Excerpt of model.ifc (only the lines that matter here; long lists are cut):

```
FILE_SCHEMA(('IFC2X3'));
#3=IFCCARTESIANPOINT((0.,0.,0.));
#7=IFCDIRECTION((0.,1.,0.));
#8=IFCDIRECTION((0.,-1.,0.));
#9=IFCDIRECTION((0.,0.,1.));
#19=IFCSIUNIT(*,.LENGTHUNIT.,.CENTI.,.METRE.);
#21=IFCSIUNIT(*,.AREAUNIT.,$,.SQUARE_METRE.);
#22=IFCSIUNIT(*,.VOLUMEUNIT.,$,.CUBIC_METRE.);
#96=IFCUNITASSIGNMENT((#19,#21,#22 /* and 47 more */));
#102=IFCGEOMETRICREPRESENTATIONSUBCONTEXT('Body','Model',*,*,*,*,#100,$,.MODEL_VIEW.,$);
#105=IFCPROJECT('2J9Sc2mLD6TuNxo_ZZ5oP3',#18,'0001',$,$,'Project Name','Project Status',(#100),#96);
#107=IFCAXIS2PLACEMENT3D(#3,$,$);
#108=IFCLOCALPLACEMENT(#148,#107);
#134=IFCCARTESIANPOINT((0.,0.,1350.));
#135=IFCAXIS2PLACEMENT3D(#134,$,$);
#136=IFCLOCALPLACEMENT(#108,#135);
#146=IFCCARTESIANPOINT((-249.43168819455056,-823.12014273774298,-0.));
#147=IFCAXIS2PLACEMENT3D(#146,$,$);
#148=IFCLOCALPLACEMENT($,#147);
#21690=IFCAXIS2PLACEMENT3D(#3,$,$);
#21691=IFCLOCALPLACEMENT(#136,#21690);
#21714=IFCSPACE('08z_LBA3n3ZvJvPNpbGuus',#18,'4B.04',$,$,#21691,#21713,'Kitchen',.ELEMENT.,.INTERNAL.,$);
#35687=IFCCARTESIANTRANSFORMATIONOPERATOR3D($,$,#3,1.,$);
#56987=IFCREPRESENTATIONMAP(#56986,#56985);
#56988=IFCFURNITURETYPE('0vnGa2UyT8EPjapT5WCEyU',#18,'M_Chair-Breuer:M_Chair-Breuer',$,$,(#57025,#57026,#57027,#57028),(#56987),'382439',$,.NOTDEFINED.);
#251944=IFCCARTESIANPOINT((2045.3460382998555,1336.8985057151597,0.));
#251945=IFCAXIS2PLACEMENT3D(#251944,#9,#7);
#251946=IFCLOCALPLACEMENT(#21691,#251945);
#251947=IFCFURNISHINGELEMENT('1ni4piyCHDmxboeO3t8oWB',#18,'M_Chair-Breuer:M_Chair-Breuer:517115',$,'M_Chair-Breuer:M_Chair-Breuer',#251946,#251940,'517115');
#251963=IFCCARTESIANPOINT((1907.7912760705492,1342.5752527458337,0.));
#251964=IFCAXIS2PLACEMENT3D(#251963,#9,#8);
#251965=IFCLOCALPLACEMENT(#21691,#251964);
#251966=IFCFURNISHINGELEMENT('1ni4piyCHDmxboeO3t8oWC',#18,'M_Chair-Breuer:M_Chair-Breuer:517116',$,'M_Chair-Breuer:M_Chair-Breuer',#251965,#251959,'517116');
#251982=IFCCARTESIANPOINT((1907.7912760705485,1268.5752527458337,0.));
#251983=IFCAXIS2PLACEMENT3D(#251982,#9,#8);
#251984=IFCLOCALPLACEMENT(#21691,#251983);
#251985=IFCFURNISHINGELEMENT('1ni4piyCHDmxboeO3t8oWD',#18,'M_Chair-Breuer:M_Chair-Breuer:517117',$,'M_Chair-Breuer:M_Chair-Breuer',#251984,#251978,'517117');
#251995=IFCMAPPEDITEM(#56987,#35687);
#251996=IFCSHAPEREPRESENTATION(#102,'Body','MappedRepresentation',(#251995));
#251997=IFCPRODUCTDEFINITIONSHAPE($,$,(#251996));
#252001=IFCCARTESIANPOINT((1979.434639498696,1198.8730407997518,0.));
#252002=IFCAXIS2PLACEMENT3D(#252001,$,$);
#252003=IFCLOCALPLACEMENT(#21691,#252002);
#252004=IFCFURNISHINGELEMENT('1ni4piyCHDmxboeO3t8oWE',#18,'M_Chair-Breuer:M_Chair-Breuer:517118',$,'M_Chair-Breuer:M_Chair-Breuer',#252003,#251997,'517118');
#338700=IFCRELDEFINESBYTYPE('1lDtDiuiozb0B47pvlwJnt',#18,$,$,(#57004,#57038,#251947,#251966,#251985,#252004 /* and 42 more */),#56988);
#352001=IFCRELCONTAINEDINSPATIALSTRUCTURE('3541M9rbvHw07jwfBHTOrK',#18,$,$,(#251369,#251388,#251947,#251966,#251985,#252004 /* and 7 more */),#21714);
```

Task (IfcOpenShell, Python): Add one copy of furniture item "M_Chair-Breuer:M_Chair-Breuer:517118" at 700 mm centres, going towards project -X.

```python
import numpy as np
import ifcopenshell
import ifcopenshell.api.geometry
import ifcopenshell.api.root
import ifcopenshell.util.element
import ifcopenshell.util.placement
import ifcopenshell.util.unit

model = ifcopenshell.open("model.ifc")
unit_scale = ifcopenshell.util.unit.calculate_unit_scale(model)


def reuse_history(source, copy):
    """copy_class also copies each property set's owner history, people and application; keep the originals."""
    for rel in copy.IsDefinedBy:
        if rel.is_a("IfcRelDefinesByProperties") and (history := rel.RelatingPropertyDefinition.OwnerHistory):
            rel.RelatingPropertyDefinition.OwnerHistory = source.OwnerHistory
            ifcopenshell.util.element.remove_deep2(model, history)


source = model.by_guid("1ni4piyCHDmxboeO3t8oWE")
base = ifcopenshell.util.placement.get_local_placement(source.ObjectPlacement)
step = np.array([-1.0, 0.0, 0.0]) * 0.7 / unit_scale

for i in range(1, 2):
    copy = ifcopenshell.api.root.copy_class(model, product=source)
    copy.Representation = ifcopenshell.util.element.copy_deep(
        model, source.Representation, exclude=["IfcGeometricRepresentationContext", "IfcRepresentationMap"]
    )
    copy.Name = "M_Chair-Breuer:M_Chair-Breuer"
    copy.Tag = None
    reuse_history(source, copy)
    matrix = base.copy()
    matrix[:3, 3] += i * step
    print("added at", matrix[:3, 3].round(3) + 0.0)
    ifcopenshell.api.geometry.edit_object_placement(model, product=copy, matrix=matrix, is_si=False)

model.write("model_updated.ifc")
```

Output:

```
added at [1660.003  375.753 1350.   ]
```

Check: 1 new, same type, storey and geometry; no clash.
